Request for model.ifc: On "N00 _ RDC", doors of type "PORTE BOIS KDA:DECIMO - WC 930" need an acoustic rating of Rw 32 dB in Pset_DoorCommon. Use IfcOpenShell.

First a look at what the model holds.

```python
import ifcopenshell
import ifcopenshell.util.element

model = ifcopenshell.open("model.ifc")
print(model.schema)
storey = next(s for s in model.by_type("IfcBuildingStorey") if s.Name == "N00 _ RDC")
doors = [e for e in ifcopenshell.util.element.get_decomposition(storey) if e.is_a("IfcDoor")]
seen = {}
for e in doors:
    element_type = ifcopenshell.util.element.get_type(e)
    key = (element_type.Name if element_type != e and element_type else None, ifcopenshell.util.element.get_pset(e, "Pset_DoorCommon", "AcousticRating"))
    seen[key] = seen.get(key, 0) + 1
for (name, value), count in sorted(seen.items(), key=str):
    print(count, "x", name, "|", value)
```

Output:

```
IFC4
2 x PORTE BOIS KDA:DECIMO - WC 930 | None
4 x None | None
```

```python
import ifcopenshell
import ifcopenshell.api.pset
import ifcopenshell.util.element

model = ifcopenshell.open("model.ifc")

storey = next(s for s in model.by_type("IfcBuildingStorey") if s.Name == "N00 _ RDC")
doors = [e for e in ifcopenshell.util.element.get_decomposition(storey) if e.is_a("IfcDoor")]

count = 0
for e in doors:
    element_type = ifcopenshell.util.element.get_type(e)
    if element_type in (None, e) or element_type.Name != "PORTE BOIS KDA:DECIMO - WC 930":
        continue
    # add_pset returns the element's existing set when there is one.
    pset = ifcopenshell.api.pset.add_pset(model, product=e, name="Pset_DoorCommon")
    ifcopenshell.api.pset.edit_pset(model, pset=pset, properties={"AcousticRating": "Rw 32 dB"})
    count += 1

print(count, "doors updated")

model.write("model_rev.ifc")
```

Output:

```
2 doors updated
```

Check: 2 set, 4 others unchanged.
